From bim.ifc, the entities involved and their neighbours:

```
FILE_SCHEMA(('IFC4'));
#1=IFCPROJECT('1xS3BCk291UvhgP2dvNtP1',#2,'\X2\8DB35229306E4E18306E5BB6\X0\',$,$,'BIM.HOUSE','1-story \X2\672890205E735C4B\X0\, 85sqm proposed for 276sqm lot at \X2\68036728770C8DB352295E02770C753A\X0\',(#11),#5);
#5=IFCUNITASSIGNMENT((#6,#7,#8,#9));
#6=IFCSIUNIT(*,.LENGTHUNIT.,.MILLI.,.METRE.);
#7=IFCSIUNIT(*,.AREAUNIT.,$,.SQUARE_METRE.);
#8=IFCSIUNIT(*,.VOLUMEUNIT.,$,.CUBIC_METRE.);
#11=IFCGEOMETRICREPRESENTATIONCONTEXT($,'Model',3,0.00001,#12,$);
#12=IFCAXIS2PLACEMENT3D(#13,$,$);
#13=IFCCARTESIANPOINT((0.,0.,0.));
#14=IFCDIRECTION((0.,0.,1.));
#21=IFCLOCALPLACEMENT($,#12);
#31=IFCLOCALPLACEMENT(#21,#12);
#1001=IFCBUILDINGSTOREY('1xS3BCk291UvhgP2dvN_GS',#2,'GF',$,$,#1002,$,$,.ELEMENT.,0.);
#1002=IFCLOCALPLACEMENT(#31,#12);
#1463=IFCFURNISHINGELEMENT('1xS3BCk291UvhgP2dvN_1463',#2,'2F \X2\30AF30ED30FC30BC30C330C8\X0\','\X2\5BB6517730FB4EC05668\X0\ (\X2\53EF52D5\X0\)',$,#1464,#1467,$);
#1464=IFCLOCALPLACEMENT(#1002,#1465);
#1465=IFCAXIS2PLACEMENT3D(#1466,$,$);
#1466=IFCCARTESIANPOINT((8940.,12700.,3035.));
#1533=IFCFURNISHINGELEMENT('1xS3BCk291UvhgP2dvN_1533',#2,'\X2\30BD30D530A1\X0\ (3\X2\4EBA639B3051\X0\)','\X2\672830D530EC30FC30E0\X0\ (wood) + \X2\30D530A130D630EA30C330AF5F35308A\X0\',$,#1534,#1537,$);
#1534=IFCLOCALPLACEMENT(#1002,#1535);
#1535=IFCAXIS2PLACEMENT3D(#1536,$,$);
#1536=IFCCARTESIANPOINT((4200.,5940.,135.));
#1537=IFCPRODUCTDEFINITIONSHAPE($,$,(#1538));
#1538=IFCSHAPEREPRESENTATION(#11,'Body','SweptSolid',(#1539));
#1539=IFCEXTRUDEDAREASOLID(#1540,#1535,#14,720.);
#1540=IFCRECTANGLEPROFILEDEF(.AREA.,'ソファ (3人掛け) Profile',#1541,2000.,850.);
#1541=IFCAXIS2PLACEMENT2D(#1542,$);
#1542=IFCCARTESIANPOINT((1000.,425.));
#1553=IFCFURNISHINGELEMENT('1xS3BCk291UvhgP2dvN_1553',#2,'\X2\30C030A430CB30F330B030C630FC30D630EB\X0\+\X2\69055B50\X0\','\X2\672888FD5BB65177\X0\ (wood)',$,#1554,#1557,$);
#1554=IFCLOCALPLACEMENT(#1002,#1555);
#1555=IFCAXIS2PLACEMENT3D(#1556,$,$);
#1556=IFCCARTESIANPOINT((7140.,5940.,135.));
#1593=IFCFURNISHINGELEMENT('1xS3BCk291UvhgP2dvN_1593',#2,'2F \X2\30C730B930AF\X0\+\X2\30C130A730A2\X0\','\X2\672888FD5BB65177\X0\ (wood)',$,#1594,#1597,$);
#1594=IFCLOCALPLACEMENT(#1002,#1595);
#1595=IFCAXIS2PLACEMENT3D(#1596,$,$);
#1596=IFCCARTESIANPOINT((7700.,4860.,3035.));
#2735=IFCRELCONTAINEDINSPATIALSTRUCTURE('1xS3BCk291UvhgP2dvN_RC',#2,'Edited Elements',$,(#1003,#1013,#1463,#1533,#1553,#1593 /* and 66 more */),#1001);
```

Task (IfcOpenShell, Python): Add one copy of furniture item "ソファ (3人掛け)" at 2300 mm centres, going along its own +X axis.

```python
import ifcopenshell
import ifcopenshell.api.geometry
import ifcopenshell.api.root
import ifcopenshell.util.element
import ifcopenshell.util.placement
import ifcopenshell.util.unit

model = ifcopenshell.open("bim.ifc")
unit_scale = ifcopenshell.util.unit.calculate_unit_scale(model)


def reuse_history(source, copy):
    """copy_class also copies each property set's owner history, people and application; keep the originals."""
    for rel in copy.IsDefinedBy:
        if rel.is_a("IfcRelDefinesByProperties") and (history := rel.RelatingPropertyDefinition.OwnerHistory):
            rel.RelatingPropertyDefinition.OwnerHistory = source.OwnerHistory
            ifcopenshell.util.element.remove_deep2(model, history)


source = model.by_id(1533)
base = ifcopenshell.util.placement.get_local_placement(source.ObjectPlacement)
step = base[:3, 0] * 2.3 / unit_scale

for i in range(1, 2):
    copy = ifcopenshell.api.root.copy_class(model, product=source)
    copy.Representation = ifcopenshell.util.element.copy_deep(
        model, source.Representation, exclude=["IfcGeometricRepresentationContext", "IfcRepresentationMap"]
    )
    reuse_history(source, copy)
    matrix = base.copy()
    matrix[:3, 3] += i * step
    print("added at", matrix[:3, 3].round(3) + 0.0)
    ifcopenshell.api.geometry.edit_object_placement(model, product=copy, matrix=matrix, is_si=False)

model.write("bim_rev.ifc")
```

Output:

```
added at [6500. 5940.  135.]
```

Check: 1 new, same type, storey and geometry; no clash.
